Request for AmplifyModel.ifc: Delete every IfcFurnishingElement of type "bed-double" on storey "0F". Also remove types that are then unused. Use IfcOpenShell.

First a look at what the model holds.

```python
import ifcopenshell
import ifcopenshell.util.element

model = ifcopenshell.open("AmplifyModel.ifc")
print(model.schema)
storey = next(s for s in model.by_type("IfcBuildingStorey") if s.Name == "0F")
furniture = [e for e in ifcopenshell.util.element.get_decomposition(storey) if e.is_a("IfcFurnishingElement")]
seen = {}
for e in furniture:
    element_type = ifcopenshell.util.element.get_type(e)
    name = element_type.Name if element_type not in (None, e) else None
    seen[name] = seen.get(name, 0) + 1
for name, count in sorted(seen.items(), key=str):
    print(count, "x", name)
```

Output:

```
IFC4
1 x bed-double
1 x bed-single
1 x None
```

```python
import ifcopenshell
import ifcopenshell.api.root
import ifcopenshell.util.element

model = ifcopenshell.open("AmplifyModel.ifc")

storey = next(s for s in model.by_type("IfcBuildingStorey") if s.Name == "0F")
furniture = [e for e in ifcopenshell.util.element.get_decomposition(storey) if e.is_a("IfcFurnishingElement")]
targets = [e for e in furniture if (t := ifcopenshell.util.element.get_type(e)) not in (None, e) and t.Name == "bed-double"]
types = {ifcopenshell.util.element.get_type(e) for e in targets} - {None, *targets}

for e in targets:
    ifcopenshell.api.root.remove_product(model, product=e)
print(len(targets), "removed")

unused = [t for t in types if not ifcopenshell.util.element.get_types(t)]
for t in unused:
    ifcopenshell.api.root.remove_product(model, product=t)
print(len(unused), "unused types removed")

model.write("AmplifyModel_v2.ifc")
```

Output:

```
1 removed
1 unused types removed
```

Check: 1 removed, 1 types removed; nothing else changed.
